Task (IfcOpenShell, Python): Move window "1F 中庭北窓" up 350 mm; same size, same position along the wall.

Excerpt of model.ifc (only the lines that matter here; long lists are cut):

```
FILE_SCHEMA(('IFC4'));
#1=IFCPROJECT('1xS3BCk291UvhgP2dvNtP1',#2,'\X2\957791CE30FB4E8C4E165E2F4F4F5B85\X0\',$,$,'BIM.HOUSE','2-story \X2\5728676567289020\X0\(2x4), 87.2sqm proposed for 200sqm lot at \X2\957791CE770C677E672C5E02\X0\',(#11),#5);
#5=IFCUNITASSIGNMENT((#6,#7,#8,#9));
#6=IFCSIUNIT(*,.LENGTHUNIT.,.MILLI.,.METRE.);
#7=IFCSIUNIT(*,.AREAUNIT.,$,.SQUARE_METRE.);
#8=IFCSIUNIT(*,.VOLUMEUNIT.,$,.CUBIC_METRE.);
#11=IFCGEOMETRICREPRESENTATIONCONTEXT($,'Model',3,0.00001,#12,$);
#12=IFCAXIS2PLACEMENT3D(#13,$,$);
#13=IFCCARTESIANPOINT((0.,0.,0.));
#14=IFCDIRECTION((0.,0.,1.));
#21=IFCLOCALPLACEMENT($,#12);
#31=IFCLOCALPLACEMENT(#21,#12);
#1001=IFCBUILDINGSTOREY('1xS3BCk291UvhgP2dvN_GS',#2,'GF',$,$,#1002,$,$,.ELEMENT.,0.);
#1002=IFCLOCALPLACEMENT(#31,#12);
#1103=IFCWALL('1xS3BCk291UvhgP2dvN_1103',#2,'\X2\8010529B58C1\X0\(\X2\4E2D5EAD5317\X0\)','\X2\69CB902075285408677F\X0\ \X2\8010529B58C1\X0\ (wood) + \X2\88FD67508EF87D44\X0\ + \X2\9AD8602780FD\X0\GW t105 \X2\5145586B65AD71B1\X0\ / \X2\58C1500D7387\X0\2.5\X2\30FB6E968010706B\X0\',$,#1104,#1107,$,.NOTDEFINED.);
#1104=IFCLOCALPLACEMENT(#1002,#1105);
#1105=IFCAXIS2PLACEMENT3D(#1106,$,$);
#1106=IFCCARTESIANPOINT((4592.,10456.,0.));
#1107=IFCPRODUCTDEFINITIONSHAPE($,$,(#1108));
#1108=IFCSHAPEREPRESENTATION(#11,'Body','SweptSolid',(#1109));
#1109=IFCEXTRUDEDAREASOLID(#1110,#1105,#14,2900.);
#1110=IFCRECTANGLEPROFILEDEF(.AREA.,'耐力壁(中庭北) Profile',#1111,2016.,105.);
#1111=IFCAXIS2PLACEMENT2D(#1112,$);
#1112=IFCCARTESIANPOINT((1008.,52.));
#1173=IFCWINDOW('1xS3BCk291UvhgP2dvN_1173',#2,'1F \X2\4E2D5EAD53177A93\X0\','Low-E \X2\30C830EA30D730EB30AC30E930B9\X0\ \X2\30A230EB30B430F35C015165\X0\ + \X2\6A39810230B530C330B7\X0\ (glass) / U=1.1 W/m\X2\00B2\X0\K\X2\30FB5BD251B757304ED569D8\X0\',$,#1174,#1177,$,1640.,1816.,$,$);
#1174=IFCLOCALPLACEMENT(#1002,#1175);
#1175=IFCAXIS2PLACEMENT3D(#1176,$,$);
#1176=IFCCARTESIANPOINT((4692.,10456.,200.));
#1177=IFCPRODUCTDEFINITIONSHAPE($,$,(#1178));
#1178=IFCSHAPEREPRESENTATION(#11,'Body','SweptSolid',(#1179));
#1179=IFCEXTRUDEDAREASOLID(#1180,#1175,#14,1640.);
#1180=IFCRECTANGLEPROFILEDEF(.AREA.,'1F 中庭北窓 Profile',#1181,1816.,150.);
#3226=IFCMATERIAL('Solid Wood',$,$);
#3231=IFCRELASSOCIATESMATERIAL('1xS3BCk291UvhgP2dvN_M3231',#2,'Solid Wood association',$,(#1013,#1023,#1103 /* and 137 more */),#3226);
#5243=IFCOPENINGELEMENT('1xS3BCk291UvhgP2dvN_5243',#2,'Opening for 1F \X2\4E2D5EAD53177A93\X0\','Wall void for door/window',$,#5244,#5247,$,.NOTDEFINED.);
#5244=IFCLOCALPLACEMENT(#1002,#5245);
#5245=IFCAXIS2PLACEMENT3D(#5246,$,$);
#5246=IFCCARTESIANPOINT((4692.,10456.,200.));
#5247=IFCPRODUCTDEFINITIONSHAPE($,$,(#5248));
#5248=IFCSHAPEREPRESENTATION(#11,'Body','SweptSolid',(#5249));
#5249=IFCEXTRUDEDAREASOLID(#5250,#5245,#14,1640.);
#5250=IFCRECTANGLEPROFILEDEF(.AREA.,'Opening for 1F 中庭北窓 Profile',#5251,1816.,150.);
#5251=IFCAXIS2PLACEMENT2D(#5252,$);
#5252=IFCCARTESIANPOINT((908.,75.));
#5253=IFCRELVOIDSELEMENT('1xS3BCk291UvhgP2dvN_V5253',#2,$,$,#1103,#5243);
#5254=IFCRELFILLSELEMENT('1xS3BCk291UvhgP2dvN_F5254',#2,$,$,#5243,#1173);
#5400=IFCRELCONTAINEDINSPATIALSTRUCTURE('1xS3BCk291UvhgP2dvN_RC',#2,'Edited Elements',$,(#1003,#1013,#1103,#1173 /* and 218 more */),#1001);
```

```python
import numpy as np
import ifcopenshell
import ifcopenshell.api.geometry
import ifcopenshell.util.placement
import ifcopenshell.util.unit

model = ifcopenshell.open("model.ifc")
unit_scale = ifcopenshell.util.unit.calculate_unit_scale(model)

window = model.by_guid("1xS3BCk291UvhgP2dvN_1173")
opening = window.FillsVoids[0].RelatingOpeningElement
dz = 0.35 / unit_scale

shift = np.array([0.0, 0.0, dz])
# The window is not placed relative to its opening, so move both.
for product in (opening, window):
    matrix = ifcopenshell.util.placement.get_local_placement(product.ObjectPlacement)
    matrix[:3, 3] += shift
    ifcopenshell.api.geometry.edit_object_placement(model, product=product, matrix=matrix, is_si=False)

print(f"moved by {dz * unit_scale:+.3f} m")

model.write("model_edited.ifc")
```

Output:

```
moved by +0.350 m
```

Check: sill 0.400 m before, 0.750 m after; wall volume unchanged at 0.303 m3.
